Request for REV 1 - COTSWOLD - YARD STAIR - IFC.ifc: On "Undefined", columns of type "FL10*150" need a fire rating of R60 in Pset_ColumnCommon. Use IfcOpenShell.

First a look at what the model holds.

```python
import ifcopenshell
import ifcopenshell.util.element

model = ifcopenshell.open("REV 1 - COTSWOLD - YARD STAIR - IFC.ifc")
print(model.schema)
storey = next(s for s in model.by_type("IfcBuildingStorey") if s.Name == "Undefined")
columns = [e for e in ifcopenshell.util.element.get_decomposition(storey) if e.is_a("IfcColumn")]
seen = {}
for e in columns:
    element_type = ifcopenshell.util.element.get_type(e)
    key = (element_type.Name if element_type != e and element_type else None, ifcopenshell.util.element.get_pset(e, "Pset_ColumnCommon", "FireRating"))
    seen[key] = seen.get(key, 0) + 1
for (name, value), count in sorted(seen.items(), key=str):
    print(count, "x", name, "|", value)
```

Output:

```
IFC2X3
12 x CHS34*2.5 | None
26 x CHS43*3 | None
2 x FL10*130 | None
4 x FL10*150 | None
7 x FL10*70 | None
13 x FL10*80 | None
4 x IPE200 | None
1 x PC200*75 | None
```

```python
import ifcopenshell
import ifcopenshell.api.pset
import ifcopenshell.util.element

model = ifcopenshell.open("REV 1 - COTSWOLD - YARD STAIR - IFC.ifc")

storey = next(s for s in model.by_type("IfcBuildingStorey") if s.Name == "Undefined")
columns = [e for e in ifcopenshell.util.element.get_decomposition(storey) if e.is_a("IfcColumn")]

count = 0
for e in columns:
    element_type = ifcopenshell.util.element.get_type(e)
    if element_type in (None, e) or element_type.Name != "FL10*150":
        continue
    found = ifcopenshell.util.element.get_pset(e, "Pset_ColumnCommon", should_inherit=False)
    if found:
        pset = model.by_id(found["id"])
        if len(ifcopenshell.util.element.get_elements_by_pset(pset)) > 1:
            pset = ifcopenshell.api.pset.unshare_pset(model, products=[e], pset=pset)[0]
    else:
        pset = ifcopenshell.api.pset.add_pset(model, product=e, name="Pset_ColumnCommon")
    ifcopenshell.api.pset.edit_pset(model, pset=pset, properties={"FireRating": "R60"})
    count += 1

print(count, "columns updated")

model.write("REV 1 - COTSWOLD - YARD STAIR - IFC_v2.ifc")
```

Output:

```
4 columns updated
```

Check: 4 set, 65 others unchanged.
